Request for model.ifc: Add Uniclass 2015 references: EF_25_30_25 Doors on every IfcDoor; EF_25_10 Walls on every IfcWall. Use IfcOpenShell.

First a look at what the model holds.

```python
import ifcopenshell

model = ifcopenshell.open("model.ifc")
print(model.schema)
print("classifications:", [c.Name for c in model.by_type("IfcClassification")])
for ifc_class in ("IfcDoor", "IfcRoof", "IfcStair", "IfcWall", "IfcWindow"):
    print(ifc_class, len(model.by_type(ifc_class)))
```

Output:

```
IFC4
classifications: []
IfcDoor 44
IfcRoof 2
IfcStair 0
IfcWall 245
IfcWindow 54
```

```python
import ifcopenshell
import ifcopenshell.api.classification

model = ifcopenshell.open("model.ifc")

system = ifcopenshell.api.classification.add_classification(model, classification="Uniclass 2015")

codes = {
    "IfcDoor": ("EF_25_30_25", "Doors"),
    "IfcWall": ("EF_25_10", "Walls"),
}
for ifc_class, (code, name) in codes.items():
    products = model.by_type(ifc_class)
    ifcopenshell.api.classification.add_reference(
        model, products=products, classification=system, identification=code, name=name
    )
    print(code, len(products))

model.write("model-out.ifc")
```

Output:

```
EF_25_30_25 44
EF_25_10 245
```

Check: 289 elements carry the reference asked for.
